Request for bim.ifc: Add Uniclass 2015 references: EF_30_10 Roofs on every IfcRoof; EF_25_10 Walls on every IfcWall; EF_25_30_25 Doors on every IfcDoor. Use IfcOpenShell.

First a look at what the model holds.

```python
import ifcopenshell

model = ifcopenshell.open("bim.ifc")
print(model.schema)
print("classifications:", [c.Name for c in model.by_type("IfcClassification")])
for ifc_class in ("IfcDoor", "IfcRoof", "IfcStair", "IfcWall", "IfcWindow"):
    print(ifc_class, len(model.by_type(ifc_class)))
```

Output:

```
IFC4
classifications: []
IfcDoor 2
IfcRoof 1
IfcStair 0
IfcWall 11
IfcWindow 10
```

```python
import ifcopenshell
import ifcopenshell.api.classification

model = ifcopenshell.open("bim.ifc")

system = ifcopenshell.api.classification.add_classification(model, classification="Uniclass 2015")

codes = {
    "IfcRoof": ("EF_30_10", "Roofs"),
    "IfcWall": ("EF_25_10", "Walls"),
    "IfcDoor": ("EF_25_30_25", "Doors"),
}
for ifc_class, (code, name) in codes.items():
    products = model.by_type(ifc_class)
    ifcopenshell.api.classification.add_reference(
        model, products=products, classification=system, identification=code, name=name
    )
    print(code, len(products))

model.write("bim_updated.ifc")
```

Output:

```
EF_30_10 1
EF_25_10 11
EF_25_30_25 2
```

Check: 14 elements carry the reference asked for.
